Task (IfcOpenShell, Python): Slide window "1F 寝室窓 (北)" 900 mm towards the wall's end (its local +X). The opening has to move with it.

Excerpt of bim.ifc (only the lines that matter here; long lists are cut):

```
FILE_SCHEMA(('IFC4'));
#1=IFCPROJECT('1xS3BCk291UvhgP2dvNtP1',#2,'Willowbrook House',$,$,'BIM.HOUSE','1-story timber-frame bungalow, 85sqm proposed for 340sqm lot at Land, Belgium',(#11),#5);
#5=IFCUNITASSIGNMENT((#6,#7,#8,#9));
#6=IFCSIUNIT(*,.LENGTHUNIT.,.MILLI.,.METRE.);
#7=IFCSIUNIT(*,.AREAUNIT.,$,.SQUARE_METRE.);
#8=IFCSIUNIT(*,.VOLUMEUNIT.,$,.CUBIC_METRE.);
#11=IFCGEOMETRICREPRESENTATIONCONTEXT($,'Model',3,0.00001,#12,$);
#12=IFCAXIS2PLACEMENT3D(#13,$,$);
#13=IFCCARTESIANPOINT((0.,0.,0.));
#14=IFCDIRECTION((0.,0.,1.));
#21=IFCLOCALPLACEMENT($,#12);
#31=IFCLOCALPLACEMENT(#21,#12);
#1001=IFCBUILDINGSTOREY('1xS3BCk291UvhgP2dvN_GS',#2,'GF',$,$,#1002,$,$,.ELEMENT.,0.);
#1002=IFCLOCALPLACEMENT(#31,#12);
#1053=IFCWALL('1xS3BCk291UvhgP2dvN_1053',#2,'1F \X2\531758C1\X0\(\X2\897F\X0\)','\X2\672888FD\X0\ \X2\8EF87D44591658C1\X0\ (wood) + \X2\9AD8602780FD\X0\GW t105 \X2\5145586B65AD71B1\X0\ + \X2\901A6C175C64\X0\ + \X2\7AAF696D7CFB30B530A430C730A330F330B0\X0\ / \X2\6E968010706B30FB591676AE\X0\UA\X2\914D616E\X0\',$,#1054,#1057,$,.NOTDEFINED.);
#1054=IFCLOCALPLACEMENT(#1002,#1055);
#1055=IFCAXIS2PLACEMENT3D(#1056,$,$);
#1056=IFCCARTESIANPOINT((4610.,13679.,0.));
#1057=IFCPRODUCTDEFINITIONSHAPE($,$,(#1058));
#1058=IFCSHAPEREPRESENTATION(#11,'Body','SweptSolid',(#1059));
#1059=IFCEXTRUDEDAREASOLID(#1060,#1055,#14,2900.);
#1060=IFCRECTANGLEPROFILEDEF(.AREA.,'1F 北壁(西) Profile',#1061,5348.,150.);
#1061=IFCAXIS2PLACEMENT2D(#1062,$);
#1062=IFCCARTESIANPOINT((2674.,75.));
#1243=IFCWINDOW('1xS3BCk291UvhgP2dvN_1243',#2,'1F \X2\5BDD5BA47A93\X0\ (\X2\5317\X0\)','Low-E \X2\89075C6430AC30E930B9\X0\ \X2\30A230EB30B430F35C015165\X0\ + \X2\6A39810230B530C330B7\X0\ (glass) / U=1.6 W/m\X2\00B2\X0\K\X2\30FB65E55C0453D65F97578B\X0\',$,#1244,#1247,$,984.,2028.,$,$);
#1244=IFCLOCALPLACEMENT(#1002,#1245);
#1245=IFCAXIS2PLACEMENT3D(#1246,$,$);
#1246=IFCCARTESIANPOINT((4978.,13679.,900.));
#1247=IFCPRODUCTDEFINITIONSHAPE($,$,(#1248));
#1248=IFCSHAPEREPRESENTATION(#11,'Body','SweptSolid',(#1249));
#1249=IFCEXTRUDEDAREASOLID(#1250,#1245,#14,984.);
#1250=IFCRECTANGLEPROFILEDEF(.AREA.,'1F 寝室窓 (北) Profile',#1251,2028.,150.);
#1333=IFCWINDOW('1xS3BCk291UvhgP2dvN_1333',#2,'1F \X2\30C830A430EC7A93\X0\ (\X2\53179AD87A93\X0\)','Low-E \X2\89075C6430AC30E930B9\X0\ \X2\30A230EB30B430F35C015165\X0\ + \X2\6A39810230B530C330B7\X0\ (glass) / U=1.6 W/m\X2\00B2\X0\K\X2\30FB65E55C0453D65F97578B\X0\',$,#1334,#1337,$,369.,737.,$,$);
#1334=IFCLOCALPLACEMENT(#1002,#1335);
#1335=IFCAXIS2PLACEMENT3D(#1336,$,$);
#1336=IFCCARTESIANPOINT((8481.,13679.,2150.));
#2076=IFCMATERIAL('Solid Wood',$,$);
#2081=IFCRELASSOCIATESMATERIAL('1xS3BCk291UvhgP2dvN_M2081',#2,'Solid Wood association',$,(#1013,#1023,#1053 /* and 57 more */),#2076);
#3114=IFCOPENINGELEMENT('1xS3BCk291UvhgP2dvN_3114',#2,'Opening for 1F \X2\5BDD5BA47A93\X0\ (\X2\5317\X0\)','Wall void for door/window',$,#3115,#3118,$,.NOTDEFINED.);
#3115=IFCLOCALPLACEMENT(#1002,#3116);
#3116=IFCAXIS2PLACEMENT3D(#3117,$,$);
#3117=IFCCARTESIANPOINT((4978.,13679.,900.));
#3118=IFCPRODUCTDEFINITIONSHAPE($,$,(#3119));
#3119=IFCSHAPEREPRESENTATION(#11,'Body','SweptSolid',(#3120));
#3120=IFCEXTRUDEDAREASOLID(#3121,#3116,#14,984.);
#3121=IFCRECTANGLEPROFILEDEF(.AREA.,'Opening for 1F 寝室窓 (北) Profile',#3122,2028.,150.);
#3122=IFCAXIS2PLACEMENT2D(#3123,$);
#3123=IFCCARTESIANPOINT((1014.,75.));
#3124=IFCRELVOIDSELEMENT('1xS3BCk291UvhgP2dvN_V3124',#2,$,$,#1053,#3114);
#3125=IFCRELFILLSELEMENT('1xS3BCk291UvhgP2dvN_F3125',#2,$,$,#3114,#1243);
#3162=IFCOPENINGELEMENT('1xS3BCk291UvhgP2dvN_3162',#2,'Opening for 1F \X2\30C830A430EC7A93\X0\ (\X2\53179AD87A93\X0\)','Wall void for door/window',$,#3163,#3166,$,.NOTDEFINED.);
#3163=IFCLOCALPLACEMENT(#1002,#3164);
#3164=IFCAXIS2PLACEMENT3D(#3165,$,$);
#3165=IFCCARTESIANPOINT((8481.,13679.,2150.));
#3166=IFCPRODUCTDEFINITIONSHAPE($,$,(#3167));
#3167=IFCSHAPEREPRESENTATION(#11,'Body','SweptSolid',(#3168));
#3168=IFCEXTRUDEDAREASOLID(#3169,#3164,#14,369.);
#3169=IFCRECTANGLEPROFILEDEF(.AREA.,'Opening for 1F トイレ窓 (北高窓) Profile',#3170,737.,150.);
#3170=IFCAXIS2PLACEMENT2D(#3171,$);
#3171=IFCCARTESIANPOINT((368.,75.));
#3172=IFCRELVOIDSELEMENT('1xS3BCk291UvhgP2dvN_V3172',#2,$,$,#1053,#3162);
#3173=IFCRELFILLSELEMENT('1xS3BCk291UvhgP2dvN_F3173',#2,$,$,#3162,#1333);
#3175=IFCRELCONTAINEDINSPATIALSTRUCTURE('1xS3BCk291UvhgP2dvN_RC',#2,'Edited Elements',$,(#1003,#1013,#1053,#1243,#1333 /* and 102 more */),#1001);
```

```python
import ifcopenshell
import ifcopenshell.api.geometry
import ifcopenshell.util.placement
import ifcopenshell.util.unit

model = ifcopenshell.open("bim.ifc")
unit_scale = ifcopenshell.util.unit.calculate_unit_scale(model)

window = model.by_id(1243)
opening = window.FillsVoids[0].RelatingOpeningElement
wall = opening.VoidsElements[0].RelatingBuildingElement

wall_matrix = ifcopenshell.util.placement.get_local_placement(wall.ObjectPlacement)
shift = wall_matrix[:3, 0] * 0.9 / unit_scale
before = ifcopenshell.util.placement.get_local_placement(window.ObjectPlacement)[:3, 3].copy()

# The window is not placed relative to its opening, so move both.
for product in (opening, window):
    matrix = ifcopenshell.util.placement.get_local_placement(product.ObjectPlacement)
    matrix[:3, 3] += shift
    ifcopenshell.api.geometry.edit_object_placement(model, product=product, matrix=matrix, is_si=False)

after = ifcopenshell.util.placement.get_local_placement(window.ObjectPlacement)[:3, 3]
print("window moved by", (after - before).round(3) + 0.0)

model.write("bim_updated.ifc")
```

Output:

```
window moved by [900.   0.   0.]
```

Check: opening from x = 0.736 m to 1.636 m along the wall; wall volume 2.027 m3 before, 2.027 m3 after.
